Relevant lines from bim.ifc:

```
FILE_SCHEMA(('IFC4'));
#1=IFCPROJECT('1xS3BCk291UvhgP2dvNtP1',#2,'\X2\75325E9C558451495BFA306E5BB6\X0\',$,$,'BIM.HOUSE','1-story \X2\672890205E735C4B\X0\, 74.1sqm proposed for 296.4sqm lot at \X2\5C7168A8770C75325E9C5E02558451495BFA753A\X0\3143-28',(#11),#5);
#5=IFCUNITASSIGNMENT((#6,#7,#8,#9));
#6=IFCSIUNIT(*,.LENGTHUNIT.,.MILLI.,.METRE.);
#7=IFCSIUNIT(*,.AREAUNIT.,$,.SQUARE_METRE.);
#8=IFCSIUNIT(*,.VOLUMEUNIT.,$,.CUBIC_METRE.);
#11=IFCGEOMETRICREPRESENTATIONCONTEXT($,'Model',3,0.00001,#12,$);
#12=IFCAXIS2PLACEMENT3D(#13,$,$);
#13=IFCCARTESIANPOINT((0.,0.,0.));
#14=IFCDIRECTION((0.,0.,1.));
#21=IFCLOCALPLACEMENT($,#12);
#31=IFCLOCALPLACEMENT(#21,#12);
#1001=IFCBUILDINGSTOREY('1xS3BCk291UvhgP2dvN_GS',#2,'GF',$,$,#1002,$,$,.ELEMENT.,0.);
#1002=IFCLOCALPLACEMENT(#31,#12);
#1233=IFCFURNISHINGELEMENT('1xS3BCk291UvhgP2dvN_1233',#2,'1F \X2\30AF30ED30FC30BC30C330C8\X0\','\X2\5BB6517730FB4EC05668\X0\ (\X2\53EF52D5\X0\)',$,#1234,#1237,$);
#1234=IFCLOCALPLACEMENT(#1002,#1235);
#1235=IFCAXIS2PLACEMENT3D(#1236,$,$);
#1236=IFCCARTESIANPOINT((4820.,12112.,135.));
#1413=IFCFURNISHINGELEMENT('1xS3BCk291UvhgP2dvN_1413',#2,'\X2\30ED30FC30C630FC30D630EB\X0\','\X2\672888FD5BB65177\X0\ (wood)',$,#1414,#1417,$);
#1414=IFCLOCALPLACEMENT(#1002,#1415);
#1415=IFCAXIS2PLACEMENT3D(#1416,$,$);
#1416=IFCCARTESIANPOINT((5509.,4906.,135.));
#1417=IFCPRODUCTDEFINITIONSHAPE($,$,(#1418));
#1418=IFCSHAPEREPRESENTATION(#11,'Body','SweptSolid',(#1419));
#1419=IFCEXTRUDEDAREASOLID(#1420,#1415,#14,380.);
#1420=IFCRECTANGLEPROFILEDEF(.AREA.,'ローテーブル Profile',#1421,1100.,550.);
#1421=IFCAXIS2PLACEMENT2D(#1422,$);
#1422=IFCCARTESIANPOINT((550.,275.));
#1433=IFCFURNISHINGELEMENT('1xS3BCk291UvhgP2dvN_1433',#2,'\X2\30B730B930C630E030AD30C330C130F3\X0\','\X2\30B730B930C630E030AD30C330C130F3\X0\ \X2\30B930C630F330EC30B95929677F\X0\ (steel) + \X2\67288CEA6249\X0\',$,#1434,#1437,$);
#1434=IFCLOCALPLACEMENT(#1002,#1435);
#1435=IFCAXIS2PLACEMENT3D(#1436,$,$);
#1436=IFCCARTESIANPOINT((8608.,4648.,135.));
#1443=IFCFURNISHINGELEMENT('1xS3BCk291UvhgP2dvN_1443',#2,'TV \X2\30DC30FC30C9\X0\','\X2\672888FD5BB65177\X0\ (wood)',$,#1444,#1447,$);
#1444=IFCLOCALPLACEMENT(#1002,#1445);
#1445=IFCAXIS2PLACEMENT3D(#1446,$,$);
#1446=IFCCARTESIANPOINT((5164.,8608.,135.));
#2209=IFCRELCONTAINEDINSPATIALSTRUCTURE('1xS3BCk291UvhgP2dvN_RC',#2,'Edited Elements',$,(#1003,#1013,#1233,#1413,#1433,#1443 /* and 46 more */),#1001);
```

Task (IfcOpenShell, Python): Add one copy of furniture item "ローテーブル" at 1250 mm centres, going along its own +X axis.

```python
import ifcopenshell
import ifcopenshell.api.geometry
import ifcopenshell.api.root
import ifcopenshell.util.element
import ifcopenshell.util.placement
import ifcopenshell.util.unit

model = ifcopenshell.open("bim.ifc")
unit_scale = ifcopenshell.util.unit.calculate_unit_scale(model)


def reuse_history(source, copy):
    """copy_class also copies each property set's owner history, people and application; keep the originals."""
    for rel in copy.IsDefinedBy:
        if rel.is_a("IfcRelDefinesByProperties") and (history := rel.RelatingPropertyDefinition.OwnerHistory):
            rel.RelatingPropertyDefinition.OwnerHistory = source.OwnerHistory
            ifcopenshell.util.element.remove_deep2(model, history)


source = model.by_id(1413)
base = ifcopenshell.util.placement.get_local_placement(source.ObjectPlacement)
step = base[:3, 0] * 1.25 / unit_scale

for i in range(1, 2):
    copy = ifcopenshell.api.root.copy_class(model, product=source)
    copy.Representation = ifcopenshell.util.element.copy_deep(
        model, source.Representation, exclude=["IfcGeometricRepresentationContext", "IfcRepresentationMap"]
    )
    reuse_history(source, copy)
    matrix = base.copy()
    matrix[:3, 3] += i * step
    print("added at", matrix[:3, 3].round(3) + 0.0)
    ifcopenshell.api.geometry.edit_object_placement(model, product=copy, matrix=matrix, is_si=False)

model.write("bim_v2.ifc")
```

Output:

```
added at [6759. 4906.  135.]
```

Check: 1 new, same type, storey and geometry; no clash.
